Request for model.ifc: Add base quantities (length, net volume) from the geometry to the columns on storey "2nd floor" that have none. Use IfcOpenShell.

First a look at what the model holds.

```python
import ifcopenshell
import ifcopenshell.util.element
import ifcopenshell.util.unit

model = ifcopenshell.open("model.ifc")
print(model.schema)
for unit_type in ("LENGTHUNIT", "AREAUNIT", "VOLUMEUNIT"):
    print(unit_type, ifcopenshell.util.unit.calculate_unit_scale(model, unit_type))
storey = next(s for s in model.by_type("IfcBuildingStorey") if s.Name == "2nd floor")
columns = [e for e in ifcopenshell.util.element.get_decomposition(storey) if e.is_a("IfcColumn")]
for e in sorted(columns, key=lambda e: e.id()):
    print(e.id(), e.is_a(), e.Name, list(ifcopenshell.util.element.get_psets(e, qtos_only=True)), sep=" | ")
```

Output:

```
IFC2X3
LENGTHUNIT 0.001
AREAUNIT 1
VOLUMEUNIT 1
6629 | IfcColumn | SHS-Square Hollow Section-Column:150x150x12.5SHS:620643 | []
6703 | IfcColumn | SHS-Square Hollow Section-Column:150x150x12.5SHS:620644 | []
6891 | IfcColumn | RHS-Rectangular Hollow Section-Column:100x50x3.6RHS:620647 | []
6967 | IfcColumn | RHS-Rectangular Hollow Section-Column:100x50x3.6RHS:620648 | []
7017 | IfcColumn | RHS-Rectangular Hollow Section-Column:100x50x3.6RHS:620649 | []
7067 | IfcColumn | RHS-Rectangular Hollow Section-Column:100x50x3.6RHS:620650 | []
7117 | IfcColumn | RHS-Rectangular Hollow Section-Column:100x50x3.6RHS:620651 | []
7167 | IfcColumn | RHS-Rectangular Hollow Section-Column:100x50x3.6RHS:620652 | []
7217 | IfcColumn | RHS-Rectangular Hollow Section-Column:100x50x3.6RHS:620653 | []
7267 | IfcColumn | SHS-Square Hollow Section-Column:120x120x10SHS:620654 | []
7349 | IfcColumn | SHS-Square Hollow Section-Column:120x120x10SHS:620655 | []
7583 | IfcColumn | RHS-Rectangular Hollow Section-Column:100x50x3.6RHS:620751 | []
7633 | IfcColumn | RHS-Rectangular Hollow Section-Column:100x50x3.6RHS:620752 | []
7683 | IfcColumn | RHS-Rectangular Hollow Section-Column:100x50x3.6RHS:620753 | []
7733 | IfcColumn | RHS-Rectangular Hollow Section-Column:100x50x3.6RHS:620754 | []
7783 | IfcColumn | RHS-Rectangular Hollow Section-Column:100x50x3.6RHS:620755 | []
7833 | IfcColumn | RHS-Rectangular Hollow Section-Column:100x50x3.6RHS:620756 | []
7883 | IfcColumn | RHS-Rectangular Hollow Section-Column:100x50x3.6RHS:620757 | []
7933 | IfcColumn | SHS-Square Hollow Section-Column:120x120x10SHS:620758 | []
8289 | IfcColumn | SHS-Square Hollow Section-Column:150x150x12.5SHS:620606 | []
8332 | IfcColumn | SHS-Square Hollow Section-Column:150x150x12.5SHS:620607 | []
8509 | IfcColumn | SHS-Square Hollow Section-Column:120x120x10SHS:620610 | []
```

```python
import ifcopenshell
import ifcopenshell.api.pset
import ifcopenshell.geom
import ifcopenshell.util.element
import ifcopenshell.util.shape
import ifcopenshell.util.unit

model = ifcopenshell.open("model.ifc")
unit_scale = ifcopenshell.util.unit.calculate_unit_scale(model)
volume_scale = ifcopenshell.util.unit.calculate_unit_scale(model, "VOLUMEUNIT")
settings = ifcopenshell.geom.settings()

storey = next(s for s in model.by_type("IfcBuildingStorey") if s.Name == "2nd floor")
columns = [e for e in ifcopenshell.util.element.get_decomposition(storey) if e.is_a("IfcColumn")]

for e in sorted(columns, key=lambda e: e.id()):
    if ifcopenshell.util.element.get_psets(e, qtos_only=True, should_inherit=False):
        continue
    # Geometry comes back in metres, in the element's own axes.
    shape = ifcopenshell.geom.create_shape(settings, e)
    values = {
        "Length": ifcopenshell.util.shape.get_z(shape.geometry) / unit_scale,
        "NetVolume": ifcopenshell.util.shape.get_volume(shape.geometry) / volume_scale,
    }
    qto = ifcopenshell.api.pset.add_qto(model, product=e, name="BaseQuantities")
    ifcopenshell.api.pset.edit_qto(model, qto=qto, properties=values)
    print(e.id(), {k: round(v, 3) for k, v in values.items()})

model.write("model_v2.ifc")
```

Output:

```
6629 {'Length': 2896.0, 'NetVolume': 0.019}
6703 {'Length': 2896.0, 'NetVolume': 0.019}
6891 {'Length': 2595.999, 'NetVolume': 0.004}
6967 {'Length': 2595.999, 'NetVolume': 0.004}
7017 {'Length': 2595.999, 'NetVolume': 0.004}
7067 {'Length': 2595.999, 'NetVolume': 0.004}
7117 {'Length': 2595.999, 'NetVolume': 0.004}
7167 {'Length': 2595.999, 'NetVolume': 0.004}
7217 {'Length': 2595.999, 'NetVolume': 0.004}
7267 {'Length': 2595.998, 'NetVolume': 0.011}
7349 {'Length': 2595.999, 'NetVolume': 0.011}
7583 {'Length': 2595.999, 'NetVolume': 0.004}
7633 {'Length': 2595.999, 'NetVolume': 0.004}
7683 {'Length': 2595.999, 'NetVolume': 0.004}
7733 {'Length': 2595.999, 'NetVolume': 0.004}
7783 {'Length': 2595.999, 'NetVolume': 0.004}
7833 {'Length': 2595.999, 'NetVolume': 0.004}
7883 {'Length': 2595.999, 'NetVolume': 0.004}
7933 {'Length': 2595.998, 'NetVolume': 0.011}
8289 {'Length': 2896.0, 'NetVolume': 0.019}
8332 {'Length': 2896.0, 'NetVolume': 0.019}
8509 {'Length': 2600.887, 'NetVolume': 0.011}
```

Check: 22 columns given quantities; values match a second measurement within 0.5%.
